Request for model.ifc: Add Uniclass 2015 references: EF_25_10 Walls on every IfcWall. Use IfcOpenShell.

First a look at what the model holds.

```python
import ifcopenshell

model = ifcopenshell.open("model.ifc")
print(model.schema)
print("classifications:", [c.Name for c in model.by_type("IfcClassification")])
for ifc_class in ("IfcDoor", "IfcRoof", "IfcStair", "IfcWall", "IfcWindow"):
    print(ifc_class, len(model.by_type(ifc_class)))
```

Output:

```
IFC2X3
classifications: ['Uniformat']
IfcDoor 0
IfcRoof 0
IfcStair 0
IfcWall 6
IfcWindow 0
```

```python
import ifcopenshell
import ifcopenshell.api.classification

model = ifcopenshell.open("model.ifc")

# IFC2X3 requires Source and Edition and has no link from the project to the system.
system = model.create_entity("IfcClassification", Source="NBS", Edition="2015", Name="Uniclass 2015")

codes = {
    "IfcWall": ("EF_25_10", "Walls"),
}
for ifc_class, (code, name) in codes.items():
    products = model.by_type(ifc_class)
    ifcopenshell.api.classification.add_reference(
        model, products=products, classification=system, identification=code, name=name
    )
    print(code, len(products))

model.write("model_updated.ifc")
```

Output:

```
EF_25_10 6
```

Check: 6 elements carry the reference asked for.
